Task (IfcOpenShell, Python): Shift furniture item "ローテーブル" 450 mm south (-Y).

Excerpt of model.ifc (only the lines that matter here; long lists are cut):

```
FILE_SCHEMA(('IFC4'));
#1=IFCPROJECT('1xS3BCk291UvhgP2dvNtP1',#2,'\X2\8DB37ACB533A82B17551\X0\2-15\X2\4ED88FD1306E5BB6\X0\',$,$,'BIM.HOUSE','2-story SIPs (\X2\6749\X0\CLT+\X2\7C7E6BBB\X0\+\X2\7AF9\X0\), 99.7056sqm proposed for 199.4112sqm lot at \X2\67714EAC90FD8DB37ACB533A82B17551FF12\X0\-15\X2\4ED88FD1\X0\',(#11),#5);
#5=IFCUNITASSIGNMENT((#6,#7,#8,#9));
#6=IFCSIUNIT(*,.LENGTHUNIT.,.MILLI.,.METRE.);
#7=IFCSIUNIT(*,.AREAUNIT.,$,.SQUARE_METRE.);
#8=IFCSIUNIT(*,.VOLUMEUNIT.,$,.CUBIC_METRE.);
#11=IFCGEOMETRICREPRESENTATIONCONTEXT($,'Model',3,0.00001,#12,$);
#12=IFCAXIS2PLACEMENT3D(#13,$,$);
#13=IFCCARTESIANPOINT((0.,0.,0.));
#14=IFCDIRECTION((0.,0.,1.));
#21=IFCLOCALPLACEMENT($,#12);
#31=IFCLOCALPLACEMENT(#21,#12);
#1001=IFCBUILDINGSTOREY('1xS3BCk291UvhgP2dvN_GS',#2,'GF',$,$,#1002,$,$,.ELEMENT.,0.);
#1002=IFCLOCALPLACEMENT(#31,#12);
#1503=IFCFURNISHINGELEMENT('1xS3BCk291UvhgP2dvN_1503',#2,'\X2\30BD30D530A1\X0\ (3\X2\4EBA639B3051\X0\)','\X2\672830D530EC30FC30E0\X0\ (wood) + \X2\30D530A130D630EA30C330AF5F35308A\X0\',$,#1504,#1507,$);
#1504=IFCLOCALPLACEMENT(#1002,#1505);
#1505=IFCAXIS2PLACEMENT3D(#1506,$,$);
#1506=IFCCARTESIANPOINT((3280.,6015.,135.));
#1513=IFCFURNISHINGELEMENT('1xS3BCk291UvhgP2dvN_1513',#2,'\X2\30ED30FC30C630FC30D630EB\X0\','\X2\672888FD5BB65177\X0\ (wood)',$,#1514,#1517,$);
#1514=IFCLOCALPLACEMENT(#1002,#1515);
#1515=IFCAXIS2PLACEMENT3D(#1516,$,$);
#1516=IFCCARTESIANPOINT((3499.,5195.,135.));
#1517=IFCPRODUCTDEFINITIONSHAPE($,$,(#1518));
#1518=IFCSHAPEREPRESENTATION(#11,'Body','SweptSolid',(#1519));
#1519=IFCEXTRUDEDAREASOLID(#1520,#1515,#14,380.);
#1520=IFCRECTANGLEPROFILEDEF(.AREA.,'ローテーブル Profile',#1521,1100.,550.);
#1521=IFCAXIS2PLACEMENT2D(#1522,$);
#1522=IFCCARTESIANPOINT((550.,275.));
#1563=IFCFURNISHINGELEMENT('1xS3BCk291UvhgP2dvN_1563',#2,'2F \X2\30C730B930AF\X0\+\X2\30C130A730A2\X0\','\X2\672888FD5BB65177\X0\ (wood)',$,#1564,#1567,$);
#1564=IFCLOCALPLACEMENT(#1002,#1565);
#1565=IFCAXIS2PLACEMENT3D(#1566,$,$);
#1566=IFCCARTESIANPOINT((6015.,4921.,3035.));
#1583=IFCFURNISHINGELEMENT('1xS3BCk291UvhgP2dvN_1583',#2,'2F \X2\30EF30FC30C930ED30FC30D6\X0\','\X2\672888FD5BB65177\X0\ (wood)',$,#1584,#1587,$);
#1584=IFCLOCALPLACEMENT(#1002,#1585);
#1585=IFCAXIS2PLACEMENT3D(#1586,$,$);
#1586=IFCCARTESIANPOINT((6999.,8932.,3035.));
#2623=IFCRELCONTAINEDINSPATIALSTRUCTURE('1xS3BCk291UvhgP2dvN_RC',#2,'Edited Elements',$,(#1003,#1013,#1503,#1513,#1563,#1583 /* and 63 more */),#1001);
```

```python
import ifcopenshell
import ifcopenshell.api.geometry
import ifcopenshell.util.placement
import ifcopenshell.util.unit

model = ifcopenshell.open("model.ifc")
unit_scale = ifcopenshell.util.unit.calculate_unit_scale(model)

item = model.by_guid("1xS3BCk291UvhgP2dvN_1513")
matrix = ifcopenshell.util.placement.get_local_placement(item.ObjectPlacement)
matrix[1, 3] -= 0.45 / unit_scale
ifcopenshell.api.geometry.edit_object_placement(model, product=item, matrix=matrix, is_si=False)

print(ifcopenshell.util.placement.get_local_placement(item.ObjectPlacement).round(3) + 0.0)

model.write("model_rev.ifc")
```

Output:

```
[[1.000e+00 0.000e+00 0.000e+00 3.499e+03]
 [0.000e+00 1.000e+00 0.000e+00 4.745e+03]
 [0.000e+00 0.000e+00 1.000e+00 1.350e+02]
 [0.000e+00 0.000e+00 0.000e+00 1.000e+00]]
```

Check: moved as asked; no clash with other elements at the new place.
